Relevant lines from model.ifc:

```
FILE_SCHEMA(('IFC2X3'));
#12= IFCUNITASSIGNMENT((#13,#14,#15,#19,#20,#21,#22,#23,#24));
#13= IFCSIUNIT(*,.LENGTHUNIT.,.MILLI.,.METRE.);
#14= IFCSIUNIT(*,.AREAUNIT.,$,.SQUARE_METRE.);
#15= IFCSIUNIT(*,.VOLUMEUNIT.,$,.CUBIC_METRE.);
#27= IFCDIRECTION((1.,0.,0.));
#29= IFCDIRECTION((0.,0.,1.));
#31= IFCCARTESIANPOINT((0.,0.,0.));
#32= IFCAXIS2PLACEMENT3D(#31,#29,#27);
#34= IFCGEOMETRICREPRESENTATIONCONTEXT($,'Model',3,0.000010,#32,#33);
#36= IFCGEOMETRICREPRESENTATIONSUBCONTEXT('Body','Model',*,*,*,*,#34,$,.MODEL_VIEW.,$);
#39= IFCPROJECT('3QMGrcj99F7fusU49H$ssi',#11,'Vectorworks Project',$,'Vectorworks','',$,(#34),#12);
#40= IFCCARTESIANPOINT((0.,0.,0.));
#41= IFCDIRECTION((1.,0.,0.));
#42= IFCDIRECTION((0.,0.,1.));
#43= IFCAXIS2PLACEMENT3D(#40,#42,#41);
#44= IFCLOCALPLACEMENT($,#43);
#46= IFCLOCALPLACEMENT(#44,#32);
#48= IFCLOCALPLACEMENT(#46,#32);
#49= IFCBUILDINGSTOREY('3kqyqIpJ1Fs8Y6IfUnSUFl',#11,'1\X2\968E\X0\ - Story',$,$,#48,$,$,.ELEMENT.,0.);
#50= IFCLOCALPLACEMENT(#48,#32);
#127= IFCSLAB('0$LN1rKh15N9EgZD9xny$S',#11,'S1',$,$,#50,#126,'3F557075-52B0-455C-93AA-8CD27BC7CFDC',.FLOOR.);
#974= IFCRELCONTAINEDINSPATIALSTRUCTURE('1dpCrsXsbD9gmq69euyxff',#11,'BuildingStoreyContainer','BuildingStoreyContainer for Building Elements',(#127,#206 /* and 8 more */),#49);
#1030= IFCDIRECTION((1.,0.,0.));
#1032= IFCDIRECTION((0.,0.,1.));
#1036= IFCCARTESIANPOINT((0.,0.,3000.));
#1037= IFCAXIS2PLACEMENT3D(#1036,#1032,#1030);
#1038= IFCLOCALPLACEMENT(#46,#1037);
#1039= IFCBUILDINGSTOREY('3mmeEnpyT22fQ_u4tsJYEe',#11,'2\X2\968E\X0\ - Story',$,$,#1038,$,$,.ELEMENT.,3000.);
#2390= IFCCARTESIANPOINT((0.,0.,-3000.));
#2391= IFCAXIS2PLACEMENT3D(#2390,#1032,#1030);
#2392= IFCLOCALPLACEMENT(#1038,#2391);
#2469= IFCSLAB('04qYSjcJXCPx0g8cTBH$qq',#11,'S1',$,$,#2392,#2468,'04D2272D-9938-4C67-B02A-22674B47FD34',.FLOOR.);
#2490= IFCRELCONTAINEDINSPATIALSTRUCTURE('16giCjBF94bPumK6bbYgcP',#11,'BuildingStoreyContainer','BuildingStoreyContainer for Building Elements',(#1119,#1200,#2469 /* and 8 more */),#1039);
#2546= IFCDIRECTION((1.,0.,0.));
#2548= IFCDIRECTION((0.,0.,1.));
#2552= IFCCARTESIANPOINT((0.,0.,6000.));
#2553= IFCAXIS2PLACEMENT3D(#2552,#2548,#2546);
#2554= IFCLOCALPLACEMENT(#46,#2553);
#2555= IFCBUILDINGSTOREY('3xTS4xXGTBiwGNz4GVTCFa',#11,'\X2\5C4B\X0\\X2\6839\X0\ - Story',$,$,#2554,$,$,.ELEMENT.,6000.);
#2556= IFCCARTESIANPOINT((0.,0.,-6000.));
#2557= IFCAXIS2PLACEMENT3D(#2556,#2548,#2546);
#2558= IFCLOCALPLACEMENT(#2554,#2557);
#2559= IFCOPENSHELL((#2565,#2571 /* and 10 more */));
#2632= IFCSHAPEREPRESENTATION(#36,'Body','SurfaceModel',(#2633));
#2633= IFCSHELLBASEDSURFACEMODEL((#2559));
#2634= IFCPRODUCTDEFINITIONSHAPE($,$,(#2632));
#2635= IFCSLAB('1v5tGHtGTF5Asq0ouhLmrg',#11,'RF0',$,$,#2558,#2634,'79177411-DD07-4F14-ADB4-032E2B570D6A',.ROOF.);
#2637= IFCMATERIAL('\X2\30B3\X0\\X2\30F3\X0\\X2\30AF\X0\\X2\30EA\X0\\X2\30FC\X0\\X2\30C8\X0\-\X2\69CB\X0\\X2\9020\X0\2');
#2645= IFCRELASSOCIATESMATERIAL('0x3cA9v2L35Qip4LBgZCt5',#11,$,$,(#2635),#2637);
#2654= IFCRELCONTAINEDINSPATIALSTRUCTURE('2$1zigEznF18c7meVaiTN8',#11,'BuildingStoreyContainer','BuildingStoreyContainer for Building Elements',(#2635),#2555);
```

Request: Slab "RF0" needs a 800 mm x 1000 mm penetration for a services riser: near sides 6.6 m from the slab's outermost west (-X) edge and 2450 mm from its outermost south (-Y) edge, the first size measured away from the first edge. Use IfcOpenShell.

```python
import numpy as np
import ifcopenshell
import ifcopenshell.api.feature
import ifcopenshell.api.geometry
import ifcopenshell.api.root
import ifcopenshell.geom
import ifcopenshell.util.placement
import ifcopenshell.util.representation
import ifcopenshell.util.shape
import ifcopenshell.util.unit

model = ifcopenshell.open("model.ifc")
unit_scale = ifcopenshell.util.unit.calculate_unit_scale(model)
settings = ifcopenshell.geom.settings()


def volume(element):
    """Net volume in cubic metres, openings subtracted."""
    shape = ifcopenshell.geom.create_shape(settings, element)
    return ifcopenshell.util.shape.get_volume(shape.geometry)


slab = model.by_guid("1v5tGHtGTF5Asq0ouhLmrg")
before = volume(slab)

# Extent in the slab's own axes, in metres. The edges named are its -X and -Y sides.
slab_shape = ifcopenshell.geom.create_shape(settings, slab)
vertices = ifcopenshell.util.shape.get_vertices(slab_shape.geometry)
x_min, y_min, bottom = vertices.min(axis=0)
top = vertices[:, 2].max()

opening = ifcopenshell.api.root.create_entity(model, ifc_class="IfcOpeningElement", name="Services riser opening")
context = ifcopenshell.util.representation.get_context(model, "Model", "Body", "MODEL_VIEW")
width, depth = 0.8, 1
outline = [(0.0, 0.0), (width, 0.0), (width, depth), (0.0, depth), (0.0, 0.0)]
# Overshoot both faces by 50 mm so the cut is clean.
shape = ifcopenshell.api.geometry.add_slab_representation(
    model, context=context, depth=top - bottom + 0.1, polyline=outline
)
ifcopenshell.api.geometry.assign_representation(model, product=opening, representation=shape)

matrix = ifcopenshell.util.placement.get_local_placement(slab.ObjectPlacement)
matrix[:, 3] = matrix @ np.append(np.array([x_min + 6.6, y_min + 2.45, bottom - 0.05]) / unit_scale, 1.0)
ifcopenshell.api.geometry.edit_object_placement(model, product=opening, matrix=matrix, is_si=False)
ifcopenshell.api.feature.add_feature(model, feature=opening, element=slab)

after = volume(slab)

print(f"slab volume {before:.3f} -> {after:.3f} m3")

model.write("model_rev.ifc")
```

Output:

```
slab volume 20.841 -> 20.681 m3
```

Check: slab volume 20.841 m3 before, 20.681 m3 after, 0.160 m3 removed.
